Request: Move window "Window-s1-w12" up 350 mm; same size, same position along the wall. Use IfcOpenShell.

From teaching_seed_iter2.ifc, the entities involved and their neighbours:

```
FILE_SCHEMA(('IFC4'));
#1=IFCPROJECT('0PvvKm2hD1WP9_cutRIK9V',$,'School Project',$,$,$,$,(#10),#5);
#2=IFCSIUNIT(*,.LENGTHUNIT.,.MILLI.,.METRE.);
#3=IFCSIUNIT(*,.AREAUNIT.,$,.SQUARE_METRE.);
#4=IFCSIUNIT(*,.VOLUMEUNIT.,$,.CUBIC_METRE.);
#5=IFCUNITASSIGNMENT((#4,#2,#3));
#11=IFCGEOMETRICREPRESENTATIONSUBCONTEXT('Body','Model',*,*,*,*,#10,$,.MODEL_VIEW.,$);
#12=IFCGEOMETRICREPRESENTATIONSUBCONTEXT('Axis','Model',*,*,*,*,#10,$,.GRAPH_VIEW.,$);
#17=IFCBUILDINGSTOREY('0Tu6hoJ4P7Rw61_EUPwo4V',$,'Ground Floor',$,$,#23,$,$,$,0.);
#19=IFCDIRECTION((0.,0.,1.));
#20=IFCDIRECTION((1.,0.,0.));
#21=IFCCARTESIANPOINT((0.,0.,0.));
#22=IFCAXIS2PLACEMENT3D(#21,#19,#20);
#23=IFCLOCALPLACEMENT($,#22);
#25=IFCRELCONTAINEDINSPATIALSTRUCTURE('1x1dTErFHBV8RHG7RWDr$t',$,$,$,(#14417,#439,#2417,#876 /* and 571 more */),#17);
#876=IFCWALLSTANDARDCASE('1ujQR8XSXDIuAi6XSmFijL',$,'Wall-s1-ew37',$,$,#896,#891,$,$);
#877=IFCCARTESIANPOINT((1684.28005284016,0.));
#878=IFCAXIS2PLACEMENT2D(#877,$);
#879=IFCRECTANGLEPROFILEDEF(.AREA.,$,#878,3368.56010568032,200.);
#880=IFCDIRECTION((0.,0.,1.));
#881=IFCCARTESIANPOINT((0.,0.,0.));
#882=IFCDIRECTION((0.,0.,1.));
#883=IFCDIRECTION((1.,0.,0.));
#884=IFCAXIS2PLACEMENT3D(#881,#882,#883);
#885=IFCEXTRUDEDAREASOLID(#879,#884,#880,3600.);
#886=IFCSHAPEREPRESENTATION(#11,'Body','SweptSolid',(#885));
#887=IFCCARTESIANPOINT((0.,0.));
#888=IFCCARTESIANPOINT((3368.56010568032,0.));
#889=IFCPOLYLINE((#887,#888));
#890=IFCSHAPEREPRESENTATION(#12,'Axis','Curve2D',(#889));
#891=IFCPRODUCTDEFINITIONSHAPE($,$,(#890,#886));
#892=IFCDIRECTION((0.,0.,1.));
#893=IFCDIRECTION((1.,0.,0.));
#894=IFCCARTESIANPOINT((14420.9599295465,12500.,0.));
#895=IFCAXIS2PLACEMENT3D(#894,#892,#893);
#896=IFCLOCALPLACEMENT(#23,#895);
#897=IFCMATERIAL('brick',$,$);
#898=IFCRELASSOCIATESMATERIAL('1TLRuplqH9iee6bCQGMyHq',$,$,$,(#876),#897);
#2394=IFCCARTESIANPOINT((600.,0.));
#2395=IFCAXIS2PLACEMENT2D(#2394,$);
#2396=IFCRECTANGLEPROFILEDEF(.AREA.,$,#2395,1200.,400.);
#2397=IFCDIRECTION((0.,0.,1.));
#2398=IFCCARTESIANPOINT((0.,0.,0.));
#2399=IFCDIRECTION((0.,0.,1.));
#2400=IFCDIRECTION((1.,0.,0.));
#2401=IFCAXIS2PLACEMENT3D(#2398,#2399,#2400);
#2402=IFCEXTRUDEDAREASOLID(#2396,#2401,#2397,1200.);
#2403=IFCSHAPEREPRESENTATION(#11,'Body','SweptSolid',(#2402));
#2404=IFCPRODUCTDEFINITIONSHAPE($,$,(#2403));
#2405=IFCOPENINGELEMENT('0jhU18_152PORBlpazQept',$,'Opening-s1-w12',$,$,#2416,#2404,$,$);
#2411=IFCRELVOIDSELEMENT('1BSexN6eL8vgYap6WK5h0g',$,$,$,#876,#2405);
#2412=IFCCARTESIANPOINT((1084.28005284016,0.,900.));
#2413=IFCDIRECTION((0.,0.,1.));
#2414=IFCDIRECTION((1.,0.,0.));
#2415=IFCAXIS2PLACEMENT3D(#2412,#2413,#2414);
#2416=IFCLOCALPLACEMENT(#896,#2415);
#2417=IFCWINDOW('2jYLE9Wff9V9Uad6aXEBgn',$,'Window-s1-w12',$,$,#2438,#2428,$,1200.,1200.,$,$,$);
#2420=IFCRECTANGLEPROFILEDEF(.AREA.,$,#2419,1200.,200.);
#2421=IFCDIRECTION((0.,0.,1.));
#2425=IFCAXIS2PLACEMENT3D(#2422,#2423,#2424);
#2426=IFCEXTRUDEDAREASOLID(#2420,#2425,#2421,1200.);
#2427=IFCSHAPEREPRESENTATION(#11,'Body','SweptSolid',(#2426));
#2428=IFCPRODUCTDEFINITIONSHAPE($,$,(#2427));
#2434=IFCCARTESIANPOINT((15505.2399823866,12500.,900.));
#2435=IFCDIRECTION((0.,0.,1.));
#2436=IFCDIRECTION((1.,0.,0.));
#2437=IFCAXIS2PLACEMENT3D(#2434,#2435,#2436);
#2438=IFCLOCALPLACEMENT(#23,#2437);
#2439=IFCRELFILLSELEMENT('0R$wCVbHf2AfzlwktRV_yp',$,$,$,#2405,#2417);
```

```python
import numpy as np
import ifcopenshell
import ifcopenshell.api.geometry
import ifcopenshell.util.placement
import ifcopenshell.util.unit

model = ifcopenshell.open("teaching_seed_iter2.ifc")
unit_scale = ifcopenshell.util.unit.calculate_unit_scale(model)

window = model.by_guid("2jYLE9Wff9V9Uad6aXEBgn")
opening = window.FillsVoids[0].RelatingOpeningElement
dz = 0.35 / unit_scale

shift = np.array([0.0, 0.0, dz])
# The window is not placed relative to its opening, so move both.
for product in (opening, window):
    matrix = ifcopenshell.util.placement.get_local_placement(product.ObjectPlacement)
    matrix[:3, 3] += shift
    ifcopenshell.api.geometry.edit_object_placement(model, product=product, matrix=matrix, is_si=False)

print(f"moved by {dz * unit_scale:+.3f} m")

model.write("teaching_seed_iter2-out.ifc")
```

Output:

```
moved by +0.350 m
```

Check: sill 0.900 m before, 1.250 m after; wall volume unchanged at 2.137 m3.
